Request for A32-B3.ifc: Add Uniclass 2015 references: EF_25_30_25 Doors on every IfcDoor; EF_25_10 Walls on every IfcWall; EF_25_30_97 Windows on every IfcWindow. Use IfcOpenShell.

First a look at what the model holds.

```python
import ifcopenshell

model = ifcopenshell.open("A32-B3.ifc")
print(model.schema)
print("classifications:", [c.Name for c in model.by_type("IfcClassification")])
for ifc_class in ("IfcDoor", "IfcRoof", "IfcStair", "IfcWall", "IfcWindow"):
    print(ifc_class, len(model.by_type(ifc_class)))
```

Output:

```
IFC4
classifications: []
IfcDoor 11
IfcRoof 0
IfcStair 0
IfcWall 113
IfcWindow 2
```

```python
import ifcopenshell
import ifcopenshell.api.classification

model = ifcopenshell.open("A32-B3.ifc")

system = ifcopenshell.api.classification.add_classification(model, classification="Uniclass 2015")

codes = {
    "IfcDoor": ("EF_25_30_25", "Doors"),
    "IfcWall": ("EF_25_10", "Walls"),
    "IfcWindow": ("EF_25_30_97", "Windows"),
}
for ifc_class, (code, name) in codes.items():
    products = model.by_type(ifc_class)
    ifcopenshell.api.classification.add_reference(
        model, products=products, classification=system, identification=code, name=name
    )
    print(code, len(products))

model.write("A32-B3_updated.ifc")
```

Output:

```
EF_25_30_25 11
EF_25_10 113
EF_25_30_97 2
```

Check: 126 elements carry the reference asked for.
